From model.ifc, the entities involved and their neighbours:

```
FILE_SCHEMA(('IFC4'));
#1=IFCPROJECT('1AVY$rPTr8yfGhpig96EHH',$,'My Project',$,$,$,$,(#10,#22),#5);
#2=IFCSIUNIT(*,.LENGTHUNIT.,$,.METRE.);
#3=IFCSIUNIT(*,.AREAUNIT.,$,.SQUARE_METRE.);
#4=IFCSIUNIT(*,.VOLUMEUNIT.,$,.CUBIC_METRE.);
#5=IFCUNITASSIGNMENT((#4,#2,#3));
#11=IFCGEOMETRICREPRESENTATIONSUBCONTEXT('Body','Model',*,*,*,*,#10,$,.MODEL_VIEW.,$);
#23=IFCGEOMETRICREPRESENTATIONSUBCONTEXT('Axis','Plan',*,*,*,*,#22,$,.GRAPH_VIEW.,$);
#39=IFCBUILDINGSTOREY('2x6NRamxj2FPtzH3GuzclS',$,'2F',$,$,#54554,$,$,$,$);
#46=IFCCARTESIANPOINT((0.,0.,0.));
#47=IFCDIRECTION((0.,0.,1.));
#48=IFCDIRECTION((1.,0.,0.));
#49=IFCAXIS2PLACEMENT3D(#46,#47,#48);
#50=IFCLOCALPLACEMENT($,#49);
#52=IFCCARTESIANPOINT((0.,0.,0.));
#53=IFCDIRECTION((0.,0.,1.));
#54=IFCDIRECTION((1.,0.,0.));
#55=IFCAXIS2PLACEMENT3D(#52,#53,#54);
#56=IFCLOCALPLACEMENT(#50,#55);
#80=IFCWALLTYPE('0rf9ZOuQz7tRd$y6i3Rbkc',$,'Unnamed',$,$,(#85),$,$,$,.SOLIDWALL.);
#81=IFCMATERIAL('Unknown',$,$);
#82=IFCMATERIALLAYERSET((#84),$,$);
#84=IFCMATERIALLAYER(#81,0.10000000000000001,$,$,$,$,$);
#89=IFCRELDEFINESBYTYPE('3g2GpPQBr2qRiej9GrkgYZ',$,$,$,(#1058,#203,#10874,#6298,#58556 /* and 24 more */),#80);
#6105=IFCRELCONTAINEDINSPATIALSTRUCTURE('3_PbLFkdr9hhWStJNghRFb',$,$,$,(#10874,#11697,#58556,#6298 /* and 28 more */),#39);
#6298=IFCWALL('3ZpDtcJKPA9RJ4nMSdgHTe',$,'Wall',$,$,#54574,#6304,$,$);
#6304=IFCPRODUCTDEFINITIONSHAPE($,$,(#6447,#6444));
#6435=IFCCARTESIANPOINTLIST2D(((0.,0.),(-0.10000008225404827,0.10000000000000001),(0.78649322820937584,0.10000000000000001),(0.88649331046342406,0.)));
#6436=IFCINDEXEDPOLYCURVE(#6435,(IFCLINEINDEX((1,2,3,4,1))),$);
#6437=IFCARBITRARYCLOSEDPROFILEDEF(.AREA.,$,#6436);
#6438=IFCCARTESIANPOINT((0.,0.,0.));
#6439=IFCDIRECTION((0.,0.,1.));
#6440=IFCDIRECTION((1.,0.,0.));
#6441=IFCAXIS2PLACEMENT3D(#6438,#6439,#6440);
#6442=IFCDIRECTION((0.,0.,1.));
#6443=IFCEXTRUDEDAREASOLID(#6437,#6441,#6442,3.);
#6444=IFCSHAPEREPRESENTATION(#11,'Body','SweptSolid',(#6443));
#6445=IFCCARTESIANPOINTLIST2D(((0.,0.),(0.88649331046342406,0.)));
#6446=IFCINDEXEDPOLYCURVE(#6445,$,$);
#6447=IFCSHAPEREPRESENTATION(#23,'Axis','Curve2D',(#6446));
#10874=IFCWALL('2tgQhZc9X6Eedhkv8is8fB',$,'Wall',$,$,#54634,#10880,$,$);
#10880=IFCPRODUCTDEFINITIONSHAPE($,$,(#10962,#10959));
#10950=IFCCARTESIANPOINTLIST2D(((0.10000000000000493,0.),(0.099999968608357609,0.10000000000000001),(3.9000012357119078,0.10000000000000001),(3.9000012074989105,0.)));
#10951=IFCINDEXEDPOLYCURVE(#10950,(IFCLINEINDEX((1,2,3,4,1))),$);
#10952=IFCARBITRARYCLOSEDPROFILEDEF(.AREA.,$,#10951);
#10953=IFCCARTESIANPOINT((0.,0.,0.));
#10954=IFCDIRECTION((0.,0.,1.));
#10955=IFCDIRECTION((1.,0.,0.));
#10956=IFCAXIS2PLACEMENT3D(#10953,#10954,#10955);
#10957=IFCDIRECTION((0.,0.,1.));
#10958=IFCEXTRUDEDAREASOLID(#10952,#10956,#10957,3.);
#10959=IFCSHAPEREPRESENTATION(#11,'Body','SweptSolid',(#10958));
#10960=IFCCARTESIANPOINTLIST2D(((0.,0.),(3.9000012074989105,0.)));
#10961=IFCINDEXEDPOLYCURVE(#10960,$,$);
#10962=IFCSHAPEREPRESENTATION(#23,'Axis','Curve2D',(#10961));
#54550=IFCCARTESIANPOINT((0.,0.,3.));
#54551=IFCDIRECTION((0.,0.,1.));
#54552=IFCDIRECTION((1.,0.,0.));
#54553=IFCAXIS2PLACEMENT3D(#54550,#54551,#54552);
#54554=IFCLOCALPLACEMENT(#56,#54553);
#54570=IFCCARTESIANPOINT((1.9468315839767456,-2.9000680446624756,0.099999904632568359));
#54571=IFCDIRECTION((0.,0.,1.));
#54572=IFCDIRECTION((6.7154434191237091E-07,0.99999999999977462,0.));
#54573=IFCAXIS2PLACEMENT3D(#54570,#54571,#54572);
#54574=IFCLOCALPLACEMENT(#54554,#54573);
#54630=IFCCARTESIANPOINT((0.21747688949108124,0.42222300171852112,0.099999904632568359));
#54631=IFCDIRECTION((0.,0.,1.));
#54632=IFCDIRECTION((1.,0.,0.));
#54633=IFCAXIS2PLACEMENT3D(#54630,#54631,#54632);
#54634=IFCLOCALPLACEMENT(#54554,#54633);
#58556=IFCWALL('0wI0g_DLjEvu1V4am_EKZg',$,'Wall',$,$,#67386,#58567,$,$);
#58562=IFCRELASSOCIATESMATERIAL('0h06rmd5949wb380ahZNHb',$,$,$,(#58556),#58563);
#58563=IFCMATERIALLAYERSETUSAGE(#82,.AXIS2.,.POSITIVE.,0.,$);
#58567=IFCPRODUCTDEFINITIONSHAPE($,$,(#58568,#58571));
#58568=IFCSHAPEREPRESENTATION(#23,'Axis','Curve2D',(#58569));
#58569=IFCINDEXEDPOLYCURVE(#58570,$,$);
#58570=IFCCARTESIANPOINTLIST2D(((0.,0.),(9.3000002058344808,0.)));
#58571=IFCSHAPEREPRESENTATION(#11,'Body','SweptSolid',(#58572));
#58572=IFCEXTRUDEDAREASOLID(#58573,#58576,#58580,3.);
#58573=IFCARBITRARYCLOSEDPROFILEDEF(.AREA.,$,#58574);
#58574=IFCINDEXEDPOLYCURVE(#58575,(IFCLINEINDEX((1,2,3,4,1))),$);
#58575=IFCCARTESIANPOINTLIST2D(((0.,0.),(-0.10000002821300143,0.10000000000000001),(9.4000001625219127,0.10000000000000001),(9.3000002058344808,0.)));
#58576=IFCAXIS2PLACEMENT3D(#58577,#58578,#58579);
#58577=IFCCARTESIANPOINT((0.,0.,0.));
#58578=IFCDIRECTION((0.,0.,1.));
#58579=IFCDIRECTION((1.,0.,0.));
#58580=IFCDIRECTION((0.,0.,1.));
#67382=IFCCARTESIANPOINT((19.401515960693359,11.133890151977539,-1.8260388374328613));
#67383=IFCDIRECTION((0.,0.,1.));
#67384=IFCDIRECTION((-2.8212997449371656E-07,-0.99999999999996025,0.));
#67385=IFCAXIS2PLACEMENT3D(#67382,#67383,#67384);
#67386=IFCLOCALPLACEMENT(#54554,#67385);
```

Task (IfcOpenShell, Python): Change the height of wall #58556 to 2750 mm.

```python
import ifcopenshell
import ifcopenshell.geom
import ifcopenshell.util.representation
import ifcopenshell.util.shape
import ifcopenshell.util.unit

model = ifcopenshell.open("model.ifc")
unit_scale = ifcopenshell.util.unit.calculate_unit_scale(model)
settings = ifcopenshell.geom.settings()


def volume(element):
    """Net volume in cubic metres, openings subtracted."""
    shape = ifcopenshell.geom.create_shape(settings, element)
    return ifcopenshell.util.shape.get_volume(shape.geometry)


wall = model.by_guid("0wI0g_DLjEvu1V4am_EKZg")
before = volume(wall)

body = ifcopenshell.util.representation.get_representation(wall, "Model", "Body")
solid = body.Items[0]
old_height = solid.Depth
solid.Depth = 2.75 / unit_scale
after = volume(wall)

print(f"height {old_height:g} -> {solid.Depth:g}, volume {before:.3f} -> {after:.3f} m3")

model.write("model_v2.ifc")
```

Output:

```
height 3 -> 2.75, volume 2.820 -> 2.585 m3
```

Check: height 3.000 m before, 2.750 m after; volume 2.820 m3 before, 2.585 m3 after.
